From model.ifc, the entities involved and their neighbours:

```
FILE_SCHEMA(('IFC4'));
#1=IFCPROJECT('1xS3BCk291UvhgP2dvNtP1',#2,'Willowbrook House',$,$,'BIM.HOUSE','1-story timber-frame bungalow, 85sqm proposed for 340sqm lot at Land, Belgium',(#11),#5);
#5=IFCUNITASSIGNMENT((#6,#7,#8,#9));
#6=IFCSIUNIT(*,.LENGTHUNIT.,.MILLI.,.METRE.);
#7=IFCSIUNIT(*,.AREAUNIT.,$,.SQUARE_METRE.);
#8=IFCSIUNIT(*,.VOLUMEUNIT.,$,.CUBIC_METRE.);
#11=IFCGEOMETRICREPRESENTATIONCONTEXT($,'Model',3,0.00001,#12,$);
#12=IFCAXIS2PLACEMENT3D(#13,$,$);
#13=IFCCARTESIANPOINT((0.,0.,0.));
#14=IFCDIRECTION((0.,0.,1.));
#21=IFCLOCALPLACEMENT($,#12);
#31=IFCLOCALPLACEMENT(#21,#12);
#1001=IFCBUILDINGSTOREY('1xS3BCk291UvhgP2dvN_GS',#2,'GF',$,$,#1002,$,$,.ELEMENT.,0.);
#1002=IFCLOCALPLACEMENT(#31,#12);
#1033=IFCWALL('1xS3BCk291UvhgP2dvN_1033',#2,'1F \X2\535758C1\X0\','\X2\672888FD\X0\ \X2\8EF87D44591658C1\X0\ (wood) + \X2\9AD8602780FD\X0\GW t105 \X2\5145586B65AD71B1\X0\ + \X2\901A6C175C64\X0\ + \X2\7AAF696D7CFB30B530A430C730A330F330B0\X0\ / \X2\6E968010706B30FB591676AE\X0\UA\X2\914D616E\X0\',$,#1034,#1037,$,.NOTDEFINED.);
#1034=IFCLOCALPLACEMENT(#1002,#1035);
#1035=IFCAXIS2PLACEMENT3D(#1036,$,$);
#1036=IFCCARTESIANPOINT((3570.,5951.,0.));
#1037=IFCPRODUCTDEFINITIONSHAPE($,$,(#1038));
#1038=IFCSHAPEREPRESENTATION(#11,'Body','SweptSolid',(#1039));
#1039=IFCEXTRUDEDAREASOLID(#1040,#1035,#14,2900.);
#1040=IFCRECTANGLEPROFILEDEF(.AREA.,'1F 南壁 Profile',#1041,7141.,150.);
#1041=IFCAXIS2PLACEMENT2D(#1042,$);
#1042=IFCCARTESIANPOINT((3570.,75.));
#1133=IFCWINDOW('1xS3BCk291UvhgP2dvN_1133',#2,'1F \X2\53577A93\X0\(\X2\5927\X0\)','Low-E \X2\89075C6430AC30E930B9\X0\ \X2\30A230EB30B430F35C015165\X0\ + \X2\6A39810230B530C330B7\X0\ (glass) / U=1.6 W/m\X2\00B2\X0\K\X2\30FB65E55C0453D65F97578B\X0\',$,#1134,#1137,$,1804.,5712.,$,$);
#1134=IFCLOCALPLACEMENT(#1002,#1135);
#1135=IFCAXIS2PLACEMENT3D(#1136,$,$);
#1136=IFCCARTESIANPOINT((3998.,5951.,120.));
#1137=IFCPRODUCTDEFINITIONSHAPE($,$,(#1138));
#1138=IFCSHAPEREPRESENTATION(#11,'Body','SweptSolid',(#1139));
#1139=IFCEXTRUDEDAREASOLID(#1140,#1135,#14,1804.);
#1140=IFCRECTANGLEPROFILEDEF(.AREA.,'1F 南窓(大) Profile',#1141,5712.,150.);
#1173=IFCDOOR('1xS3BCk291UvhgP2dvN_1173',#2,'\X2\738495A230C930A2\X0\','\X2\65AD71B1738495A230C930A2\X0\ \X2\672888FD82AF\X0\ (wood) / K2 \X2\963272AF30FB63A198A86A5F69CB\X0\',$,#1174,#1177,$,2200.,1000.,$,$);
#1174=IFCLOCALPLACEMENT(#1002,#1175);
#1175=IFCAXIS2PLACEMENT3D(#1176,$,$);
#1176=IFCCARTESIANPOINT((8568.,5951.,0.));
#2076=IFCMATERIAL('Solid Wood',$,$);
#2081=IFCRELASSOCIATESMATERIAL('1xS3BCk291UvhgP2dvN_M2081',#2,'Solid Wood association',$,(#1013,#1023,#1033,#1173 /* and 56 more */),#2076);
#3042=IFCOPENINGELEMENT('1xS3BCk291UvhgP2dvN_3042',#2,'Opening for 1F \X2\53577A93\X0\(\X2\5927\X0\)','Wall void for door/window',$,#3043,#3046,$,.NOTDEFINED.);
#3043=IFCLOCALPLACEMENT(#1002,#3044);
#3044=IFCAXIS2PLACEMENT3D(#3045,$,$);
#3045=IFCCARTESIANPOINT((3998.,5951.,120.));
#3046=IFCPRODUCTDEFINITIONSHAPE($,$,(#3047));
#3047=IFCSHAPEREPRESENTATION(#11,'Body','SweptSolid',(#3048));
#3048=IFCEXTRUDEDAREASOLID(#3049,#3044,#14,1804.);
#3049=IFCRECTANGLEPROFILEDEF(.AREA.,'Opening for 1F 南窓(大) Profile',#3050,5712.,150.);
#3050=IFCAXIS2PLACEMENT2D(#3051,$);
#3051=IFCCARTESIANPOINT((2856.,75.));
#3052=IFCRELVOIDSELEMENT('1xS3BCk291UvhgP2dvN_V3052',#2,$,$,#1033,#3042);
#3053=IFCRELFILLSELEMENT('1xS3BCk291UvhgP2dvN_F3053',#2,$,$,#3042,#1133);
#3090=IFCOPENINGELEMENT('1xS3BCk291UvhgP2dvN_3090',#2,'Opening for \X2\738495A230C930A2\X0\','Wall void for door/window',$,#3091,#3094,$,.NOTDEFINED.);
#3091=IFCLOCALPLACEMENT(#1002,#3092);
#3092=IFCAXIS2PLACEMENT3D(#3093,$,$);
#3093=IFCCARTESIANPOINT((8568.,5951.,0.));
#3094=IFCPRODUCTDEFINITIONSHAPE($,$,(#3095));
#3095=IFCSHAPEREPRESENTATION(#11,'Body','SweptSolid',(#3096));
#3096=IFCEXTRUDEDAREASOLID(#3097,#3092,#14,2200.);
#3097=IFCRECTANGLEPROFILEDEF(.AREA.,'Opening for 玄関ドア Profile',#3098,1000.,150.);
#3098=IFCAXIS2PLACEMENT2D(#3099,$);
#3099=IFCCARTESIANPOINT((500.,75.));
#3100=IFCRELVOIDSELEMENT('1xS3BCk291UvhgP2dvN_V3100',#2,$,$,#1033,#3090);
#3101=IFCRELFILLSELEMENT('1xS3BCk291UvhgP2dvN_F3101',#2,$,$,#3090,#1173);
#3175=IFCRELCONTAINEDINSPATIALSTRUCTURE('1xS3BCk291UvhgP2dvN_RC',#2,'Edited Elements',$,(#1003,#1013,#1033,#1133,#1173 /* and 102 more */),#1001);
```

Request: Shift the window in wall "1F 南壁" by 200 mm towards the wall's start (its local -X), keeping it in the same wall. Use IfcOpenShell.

```python
import ifcopenshell
import ifcopenshell.api.geometry
import ifcopenshell.util.placement
import ifcopenshell.util.unit

model = ifcopenshell.open("model.ifc")
unit_scale = ifcopenshell.util.unit.calculate_unit_scale(model)

window = model.by_guid("1xS3BCk291UvhgP2dvN_1133")
opening = window.FillsVoids[0].RelatingOpeningElement
wall = opening.VoidsElements[0].RelatingBuildingElement

wall_matrix = ifcopenshell.util.placement.get_local_placement(wall.ObjectPlacement)
shift = wall_matrix[:3, 0] * -0.2 / unit_scale
before = ifcopenshell.util.placement.get_local_placement(window.ObjectPlacement)[:3, 3].copy()

# The window is not placed relative to its opening, so move both.
for product in (opening, window):
    matrix = ifcopenshell.util.placement.get_local_placement(product.ObjectPlacement)
    matrix[:3, 3] += shift
    ifcopenshell.api.geometry.edit_object_placement(model, product=product, matrix=matrix, is_si=False)

after = ifcopenshell.util.placement.get_local_placement(window.ObjectPlacement)[:3, 3]
print("window moved by", (after - before).round(3) + 0.0)

model.write("model-out.ifc")
```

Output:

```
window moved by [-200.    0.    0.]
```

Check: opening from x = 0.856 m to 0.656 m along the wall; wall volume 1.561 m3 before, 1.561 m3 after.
